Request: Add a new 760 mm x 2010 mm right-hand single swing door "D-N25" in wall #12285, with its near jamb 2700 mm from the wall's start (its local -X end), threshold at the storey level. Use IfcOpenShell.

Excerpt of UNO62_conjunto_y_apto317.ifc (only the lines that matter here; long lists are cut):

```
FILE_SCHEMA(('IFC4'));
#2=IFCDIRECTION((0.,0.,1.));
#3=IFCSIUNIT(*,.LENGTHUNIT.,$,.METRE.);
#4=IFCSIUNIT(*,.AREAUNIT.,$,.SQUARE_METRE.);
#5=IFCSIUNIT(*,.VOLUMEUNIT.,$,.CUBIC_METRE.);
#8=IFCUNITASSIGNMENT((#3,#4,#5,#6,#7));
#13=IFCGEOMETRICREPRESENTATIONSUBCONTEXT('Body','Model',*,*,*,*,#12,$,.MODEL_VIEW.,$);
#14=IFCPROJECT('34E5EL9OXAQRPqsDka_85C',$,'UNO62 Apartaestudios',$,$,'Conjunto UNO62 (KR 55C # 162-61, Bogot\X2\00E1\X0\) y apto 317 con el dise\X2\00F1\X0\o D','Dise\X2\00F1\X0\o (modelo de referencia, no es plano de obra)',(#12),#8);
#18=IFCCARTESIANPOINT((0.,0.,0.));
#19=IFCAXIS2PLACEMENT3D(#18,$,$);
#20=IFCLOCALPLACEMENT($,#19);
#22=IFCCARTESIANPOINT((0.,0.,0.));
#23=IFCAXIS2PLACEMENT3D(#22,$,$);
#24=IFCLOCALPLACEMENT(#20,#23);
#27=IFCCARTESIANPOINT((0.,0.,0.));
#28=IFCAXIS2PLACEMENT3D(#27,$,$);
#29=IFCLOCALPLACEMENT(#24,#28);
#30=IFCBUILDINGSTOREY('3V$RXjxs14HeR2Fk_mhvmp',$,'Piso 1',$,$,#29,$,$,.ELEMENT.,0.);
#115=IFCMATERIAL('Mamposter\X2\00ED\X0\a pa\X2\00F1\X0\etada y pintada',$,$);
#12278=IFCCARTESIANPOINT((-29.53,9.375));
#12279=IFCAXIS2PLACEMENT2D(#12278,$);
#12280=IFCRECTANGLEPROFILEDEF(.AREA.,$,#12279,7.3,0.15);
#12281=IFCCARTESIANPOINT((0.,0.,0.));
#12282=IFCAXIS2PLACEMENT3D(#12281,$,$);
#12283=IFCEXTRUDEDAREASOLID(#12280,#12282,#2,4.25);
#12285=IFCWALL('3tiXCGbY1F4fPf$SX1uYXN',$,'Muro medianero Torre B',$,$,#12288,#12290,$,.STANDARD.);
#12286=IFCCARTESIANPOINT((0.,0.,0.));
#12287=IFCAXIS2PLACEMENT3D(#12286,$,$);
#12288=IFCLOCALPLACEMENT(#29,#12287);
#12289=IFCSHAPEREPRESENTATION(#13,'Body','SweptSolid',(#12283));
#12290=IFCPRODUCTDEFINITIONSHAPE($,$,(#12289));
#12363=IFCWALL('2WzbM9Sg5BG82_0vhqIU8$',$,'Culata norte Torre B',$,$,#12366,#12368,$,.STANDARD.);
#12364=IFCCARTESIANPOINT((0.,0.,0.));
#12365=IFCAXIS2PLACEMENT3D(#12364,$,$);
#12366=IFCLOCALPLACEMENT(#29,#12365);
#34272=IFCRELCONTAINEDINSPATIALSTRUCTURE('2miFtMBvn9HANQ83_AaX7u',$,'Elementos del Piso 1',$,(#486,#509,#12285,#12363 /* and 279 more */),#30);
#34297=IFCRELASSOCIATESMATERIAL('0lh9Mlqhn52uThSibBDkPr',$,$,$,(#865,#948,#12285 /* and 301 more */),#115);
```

```python
import numpy as np
import ifcopenshell
import ifcopenshell.api.feature
import ifcopenshell.api.geometry
import ifcopenshell.api.root
import ifcopenshell.api.spatial
import ifcopenshell.geom
import ifcopenshell.util.element
import ifcopenshell.util.placement
import ifcopenshell.util.representation
import ifcopenshell.util.shape
import ifcopenshell.util.unit

model = ifcopenshell.open("UNO62_conjunto_y_apto317.ifc")
unit_scale = ifcopenshell.util.unit.calculate_unit_scale(model)
settings = ifcopenshell.geom.settings()


def volume(element):
    """Net volume in cubic metres, openings subtracted."""
    shape = ifcopenshell.geom.create_shape(settings, element)
    return ifcopenshell.util.shape.get_volume(shape.geometry)


wall = model.by_id(12285)
storey = ifcopenshell.util.element.get_container(wall, ifc_class="IfcBuildingStorey")
context = ifcopenshell.util.representation.get_context(model, "Model", "Body", "MODEL_VIEW")
before = volume(wall)

width, height, from_end, sill = 0.76, 2.01, 2.7, 0.0  # metres

# The wall runs along its own X axis, and the end named is its -X end.
wall_shape = ifcopenshell.geom.create_shape(settings, wall)
x, y, z = ifcopenshell.util.shape.get_vertices(wall_shape.geometry).T
start = x.min() + from_end
face, thickness = float(y.min()), float(y.max() - y.min())
wall_matrix = ifcopenshell.util.placement.get_local_placement(wall.ObjectPlacement)
level = ifcopenshell.util.placement.get_local_placement(storey.ObjectPlacement)[2, 3]


def in_wall(x, y):
    """Placement at x, y metres in the wall's axes, at sill height."""
    matrix = wall_matrix.copy()
    matrix[:, 3] = wall_matrix @ np.array([x / unit_scale, y / unit_scale, 0.0, 1.0])
    matrix[2, 3] = level + sill / unit_scale
    return matrix


# Opening: a box that overshoots both wall faces by 50 mm.
opening = ifcopenshell.api.root.create_entity(model, ifc_class="IfcOpeningElement", predefined_type="OPENING")
box = ifcopenshell.api.geometry.add_wall_representation(
    model, context=context, length=width, height=height, thickness=thickness + 0.1
)
ifcopenshell.api.geometry.assign_representation(model, product=opening, representation=box)
ifcopenshell.api.geometry.edit_object_placement(model, product=opening, matrix=in_wall(start, face - 0.05), is_si=False)
ifcopenshell.api.feature.add_feature(model, feature=opening, element=wall)

door = ifcopenshell.api.root.create_entity(model, ifc_class="IfcDoor", name="D-N25", predefined_type="DOOR")
door.OverallWidth, door.OverallHeight = width / unit_scale, height / unit_scale
door.OperationType = "SINGLE_SWING_RIGHT"
body = ifcopenshell.api.geometry.add_door_representation(
    model,
    context=context,
    overall_width=door.OverallWidth,
    overall_height=door.OverallHeight,
    operation_type="SINGLE_SWING_RIGHT",
    lining_properties={"LiningDepth": thickness / unit_scale, "ThresholdDepth": thickness / unit_scale},
)
ifcopenshell.api.geometry.assign_representation(model, product=door, representation=body)
ifcopenshell.api.spatial.assign_container(model, products=[door], relating_structure=storey)
ifcopenshell.api.feature.add_filling(model, opening=opening, element=door)

# The lining spans the wall, so the door starts at the wall face.
ifcopenshell.api.geometry.edit_object_placement(model, product=door, matrix=in_wall(start, face), is_si=False)

after = volume(wall)

print(f"wall volume {before:.3f} -> {after:.3f} m3")

model.write("UNO62_conjunto_y_apto317_updated.ifc")
```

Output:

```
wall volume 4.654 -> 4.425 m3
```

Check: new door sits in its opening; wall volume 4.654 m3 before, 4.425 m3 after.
